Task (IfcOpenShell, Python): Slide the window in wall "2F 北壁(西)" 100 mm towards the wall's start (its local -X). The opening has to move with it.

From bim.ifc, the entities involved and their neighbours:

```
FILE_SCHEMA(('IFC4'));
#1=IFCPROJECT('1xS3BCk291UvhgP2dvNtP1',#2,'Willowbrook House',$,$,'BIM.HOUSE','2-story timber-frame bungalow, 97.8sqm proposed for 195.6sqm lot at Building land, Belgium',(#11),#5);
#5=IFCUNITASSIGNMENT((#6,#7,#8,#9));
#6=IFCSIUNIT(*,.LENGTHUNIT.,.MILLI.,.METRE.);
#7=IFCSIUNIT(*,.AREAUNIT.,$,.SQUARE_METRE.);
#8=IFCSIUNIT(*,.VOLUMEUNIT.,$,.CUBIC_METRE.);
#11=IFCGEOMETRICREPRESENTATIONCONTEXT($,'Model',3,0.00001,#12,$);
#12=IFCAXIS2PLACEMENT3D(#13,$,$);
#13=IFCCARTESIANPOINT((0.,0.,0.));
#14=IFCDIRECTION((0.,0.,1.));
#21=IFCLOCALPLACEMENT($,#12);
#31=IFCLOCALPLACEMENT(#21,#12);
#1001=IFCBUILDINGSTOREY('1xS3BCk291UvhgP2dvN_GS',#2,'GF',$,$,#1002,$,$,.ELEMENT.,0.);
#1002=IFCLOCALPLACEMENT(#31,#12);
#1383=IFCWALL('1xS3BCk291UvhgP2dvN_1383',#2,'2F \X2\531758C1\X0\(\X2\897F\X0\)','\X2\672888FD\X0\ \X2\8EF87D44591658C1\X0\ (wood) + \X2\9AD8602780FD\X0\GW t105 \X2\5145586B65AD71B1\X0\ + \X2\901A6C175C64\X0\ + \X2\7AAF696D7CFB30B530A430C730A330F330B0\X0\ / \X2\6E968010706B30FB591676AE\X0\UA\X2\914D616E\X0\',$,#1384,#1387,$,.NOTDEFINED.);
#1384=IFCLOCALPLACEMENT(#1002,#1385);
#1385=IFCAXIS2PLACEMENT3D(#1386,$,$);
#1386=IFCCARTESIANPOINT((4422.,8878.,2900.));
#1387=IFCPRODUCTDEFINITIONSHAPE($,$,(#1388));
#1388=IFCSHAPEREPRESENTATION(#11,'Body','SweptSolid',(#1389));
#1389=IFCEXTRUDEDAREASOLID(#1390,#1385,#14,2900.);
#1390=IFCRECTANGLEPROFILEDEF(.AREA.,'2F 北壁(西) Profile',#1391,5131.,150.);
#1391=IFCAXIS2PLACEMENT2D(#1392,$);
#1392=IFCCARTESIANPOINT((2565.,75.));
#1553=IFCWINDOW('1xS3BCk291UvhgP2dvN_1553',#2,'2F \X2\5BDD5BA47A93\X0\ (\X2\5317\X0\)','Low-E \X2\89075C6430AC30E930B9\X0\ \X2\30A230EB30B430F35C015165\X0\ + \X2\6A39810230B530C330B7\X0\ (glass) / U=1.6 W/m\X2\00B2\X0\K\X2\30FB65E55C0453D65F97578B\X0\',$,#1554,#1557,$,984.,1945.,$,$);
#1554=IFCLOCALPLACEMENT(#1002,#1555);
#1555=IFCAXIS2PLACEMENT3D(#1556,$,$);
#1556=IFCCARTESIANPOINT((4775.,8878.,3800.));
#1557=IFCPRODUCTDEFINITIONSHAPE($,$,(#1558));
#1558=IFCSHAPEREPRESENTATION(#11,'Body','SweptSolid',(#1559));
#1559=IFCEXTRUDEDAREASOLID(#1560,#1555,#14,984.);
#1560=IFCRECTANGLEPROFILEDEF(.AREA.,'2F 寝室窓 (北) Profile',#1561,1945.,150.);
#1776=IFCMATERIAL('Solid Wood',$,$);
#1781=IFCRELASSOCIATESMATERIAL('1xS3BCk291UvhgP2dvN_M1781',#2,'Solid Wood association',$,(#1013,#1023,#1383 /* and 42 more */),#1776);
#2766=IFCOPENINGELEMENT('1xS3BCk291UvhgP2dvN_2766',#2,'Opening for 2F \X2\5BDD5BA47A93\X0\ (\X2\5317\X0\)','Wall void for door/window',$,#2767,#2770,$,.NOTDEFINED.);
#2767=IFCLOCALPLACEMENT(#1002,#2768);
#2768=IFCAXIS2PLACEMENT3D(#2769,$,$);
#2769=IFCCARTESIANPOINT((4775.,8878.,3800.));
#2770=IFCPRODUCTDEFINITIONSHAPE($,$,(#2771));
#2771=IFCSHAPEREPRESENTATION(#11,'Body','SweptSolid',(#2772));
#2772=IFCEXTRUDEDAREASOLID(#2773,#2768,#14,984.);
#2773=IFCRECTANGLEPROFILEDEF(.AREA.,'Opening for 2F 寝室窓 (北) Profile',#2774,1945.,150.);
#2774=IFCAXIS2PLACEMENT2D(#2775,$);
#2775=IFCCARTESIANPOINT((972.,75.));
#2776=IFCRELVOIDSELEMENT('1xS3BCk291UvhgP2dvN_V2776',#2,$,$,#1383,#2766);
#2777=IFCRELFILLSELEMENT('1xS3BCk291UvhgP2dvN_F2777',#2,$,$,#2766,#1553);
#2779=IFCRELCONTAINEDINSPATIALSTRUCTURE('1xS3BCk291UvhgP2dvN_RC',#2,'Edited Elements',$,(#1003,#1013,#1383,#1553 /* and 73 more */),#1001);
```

```python
import ifcopenshell
import ifcopenshell.api.geometry
import ifcopenshell.util.placement

model = ifcopenshell.open("bim.ifc")

window = model.by_guid("1xS3BCk291UvhgP2dvN_1553")
opening = window.FillsVoids[0].RelatingOpeningElement
wall = opening.VoidsElements[0].RelatingBuildingElement

wall_matrix = ifcopenshell.util.placement.get_local_placement(wall.ObjectPlacement)
shift = wall_matrix[:3, 0] * -100.0
before = ifcopenshell.util.placement.get_local_placement(window.ObjectPlacement)[:3, 3].copy()

# The window is not placed relative to its opening, so move both.
for product in (opening, window):
    matrix = ifcopenshell.util.placement.get_local_placement(product.ObjectPlacement)
    matrix[:3, 3] += shift
    ifcopenshell.api.geometry.edit_object_placement(model, product=product, matrix=matrix, is_si=False)

after = ifcopenshell.util.placement.get_local_placement(window.ObjectPlacement)[:3, 3]
print("window moved by", (after - before).round(3) + 0.0)

model.write("bim-out.ifc")
```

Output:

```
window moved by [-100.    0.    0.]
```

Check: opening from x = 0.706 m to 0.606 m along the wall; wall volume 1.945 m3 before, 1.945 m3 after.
